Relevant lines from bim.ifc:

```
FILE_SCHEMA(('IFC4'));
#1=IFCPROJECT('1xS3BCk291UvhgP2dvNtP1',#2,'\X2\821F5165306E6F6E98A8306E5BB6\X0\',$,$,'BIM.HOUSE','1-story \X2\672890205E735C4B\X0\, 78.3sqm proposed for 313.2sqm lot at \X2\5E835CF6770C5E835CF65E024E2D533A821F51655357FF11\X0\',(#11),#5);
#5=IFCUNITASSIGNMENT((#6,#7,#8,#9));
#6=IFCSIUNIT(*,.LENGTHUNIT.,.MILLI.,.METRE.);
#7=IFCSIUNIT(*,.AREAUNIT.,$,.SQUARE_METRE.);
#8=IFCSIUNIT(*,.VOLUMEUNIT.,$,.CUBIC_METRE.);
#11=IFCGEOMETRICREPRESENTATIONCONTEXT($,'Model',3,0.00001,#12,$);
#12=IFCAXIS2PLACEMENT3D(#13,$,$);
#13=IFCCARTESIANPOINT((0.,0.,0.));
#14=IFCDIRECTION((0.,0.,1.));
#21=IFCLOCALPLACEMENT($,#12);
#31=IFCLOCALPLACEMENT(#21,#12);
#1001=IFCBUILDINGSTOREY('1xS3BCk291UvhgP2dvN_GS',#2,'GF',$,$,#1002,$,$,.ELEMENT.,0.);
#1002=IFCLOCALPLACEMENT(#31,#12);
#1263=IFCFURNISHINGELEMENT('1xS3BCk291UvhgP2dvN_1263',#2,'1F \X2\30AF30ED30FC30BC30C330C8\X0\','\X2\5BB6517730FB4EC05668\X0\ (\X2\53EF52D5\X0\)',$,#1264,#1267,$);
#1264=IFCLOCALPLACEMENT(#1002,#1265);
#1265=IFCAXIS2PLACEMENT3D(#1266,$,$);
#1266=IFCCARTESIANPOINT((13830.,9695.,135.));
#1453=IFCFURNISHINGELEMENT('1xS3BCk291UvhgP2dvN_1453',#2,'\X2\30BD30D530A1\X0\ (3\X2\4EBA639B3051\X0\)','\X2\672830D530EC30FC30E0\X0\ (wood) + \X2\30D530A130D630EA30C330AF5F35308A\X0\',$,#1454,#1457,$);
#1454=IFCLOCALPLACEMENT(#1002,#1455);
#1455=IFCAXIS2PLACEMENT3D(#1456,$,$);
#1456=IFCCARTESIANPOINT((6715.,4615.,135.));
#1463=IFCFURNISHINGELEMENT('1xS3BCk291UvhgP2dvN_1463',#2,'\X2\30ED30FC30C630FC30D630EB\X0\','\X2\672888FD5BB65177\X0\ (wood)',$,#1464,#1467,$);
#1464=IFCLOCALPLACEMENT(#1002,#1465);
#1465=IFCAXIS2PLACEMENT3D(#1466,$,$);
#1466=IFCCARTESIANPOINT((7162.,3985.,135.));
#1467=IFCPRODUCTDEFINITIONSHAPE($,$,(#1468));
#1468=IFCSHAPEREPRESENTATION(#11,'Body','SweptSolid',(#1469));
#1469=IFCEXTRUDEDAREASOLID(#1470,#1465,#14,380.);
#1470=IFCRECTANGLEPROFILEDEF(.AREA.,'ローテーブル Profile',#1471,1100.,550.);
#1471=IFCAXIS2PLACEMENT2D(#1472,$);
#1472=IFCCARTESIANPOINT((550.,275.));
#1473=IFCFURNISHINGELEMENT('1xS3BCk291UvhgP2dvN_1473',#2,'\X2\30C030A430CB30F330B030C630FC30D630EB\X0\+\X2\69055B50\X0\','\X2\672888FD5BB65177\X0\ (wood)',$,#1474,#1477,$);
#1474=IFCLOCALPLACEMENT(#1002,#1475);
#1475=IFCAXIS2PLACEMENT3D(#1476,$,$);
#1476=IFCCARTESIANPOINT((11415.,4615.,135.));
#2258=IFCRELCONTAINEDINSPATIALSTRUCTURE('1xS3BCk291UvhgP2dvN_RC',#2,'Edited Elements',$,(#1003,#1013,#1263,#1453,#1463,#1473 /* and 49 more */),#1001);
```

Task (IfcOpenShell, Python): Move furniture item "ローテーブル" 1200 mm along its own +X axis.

```python
import ifcopenshell
import ifcopenshell.api.geometry
import ifcopenshell.util.placement
import ifcopenshell.util.unit

model = ifcopenshell.open("bim.ifc")
unit_scale = ifcopenshell.util.unit.calculate_unit_scale(model)

item = model.by_guid("1xS3BCk291UvhgP2dvN_1463")
matrix = ifcopenshell.util.placement.get_local_placement(item.ObjectPlacement)
matrix[:3, 3] += matrix[:3, 0] * 1.2 / unit_scale
ifcopenshell.api.geometry.edit_object_placement(model, product=item, matrix=matrix, is_si=False)

print(ifcopenshell.util.placement.get_local_placement(item.ObjectPlacement).round(3) + 0.0)

model.write("bim_rev.ifc")
```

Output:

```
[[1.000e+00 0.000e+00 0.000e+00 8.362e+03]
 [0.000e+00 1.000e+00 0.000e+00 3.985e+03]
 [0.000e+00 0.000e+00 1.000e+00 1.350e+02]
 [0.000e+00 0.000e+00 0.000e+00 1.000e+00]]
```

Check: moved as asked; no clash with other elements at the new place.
